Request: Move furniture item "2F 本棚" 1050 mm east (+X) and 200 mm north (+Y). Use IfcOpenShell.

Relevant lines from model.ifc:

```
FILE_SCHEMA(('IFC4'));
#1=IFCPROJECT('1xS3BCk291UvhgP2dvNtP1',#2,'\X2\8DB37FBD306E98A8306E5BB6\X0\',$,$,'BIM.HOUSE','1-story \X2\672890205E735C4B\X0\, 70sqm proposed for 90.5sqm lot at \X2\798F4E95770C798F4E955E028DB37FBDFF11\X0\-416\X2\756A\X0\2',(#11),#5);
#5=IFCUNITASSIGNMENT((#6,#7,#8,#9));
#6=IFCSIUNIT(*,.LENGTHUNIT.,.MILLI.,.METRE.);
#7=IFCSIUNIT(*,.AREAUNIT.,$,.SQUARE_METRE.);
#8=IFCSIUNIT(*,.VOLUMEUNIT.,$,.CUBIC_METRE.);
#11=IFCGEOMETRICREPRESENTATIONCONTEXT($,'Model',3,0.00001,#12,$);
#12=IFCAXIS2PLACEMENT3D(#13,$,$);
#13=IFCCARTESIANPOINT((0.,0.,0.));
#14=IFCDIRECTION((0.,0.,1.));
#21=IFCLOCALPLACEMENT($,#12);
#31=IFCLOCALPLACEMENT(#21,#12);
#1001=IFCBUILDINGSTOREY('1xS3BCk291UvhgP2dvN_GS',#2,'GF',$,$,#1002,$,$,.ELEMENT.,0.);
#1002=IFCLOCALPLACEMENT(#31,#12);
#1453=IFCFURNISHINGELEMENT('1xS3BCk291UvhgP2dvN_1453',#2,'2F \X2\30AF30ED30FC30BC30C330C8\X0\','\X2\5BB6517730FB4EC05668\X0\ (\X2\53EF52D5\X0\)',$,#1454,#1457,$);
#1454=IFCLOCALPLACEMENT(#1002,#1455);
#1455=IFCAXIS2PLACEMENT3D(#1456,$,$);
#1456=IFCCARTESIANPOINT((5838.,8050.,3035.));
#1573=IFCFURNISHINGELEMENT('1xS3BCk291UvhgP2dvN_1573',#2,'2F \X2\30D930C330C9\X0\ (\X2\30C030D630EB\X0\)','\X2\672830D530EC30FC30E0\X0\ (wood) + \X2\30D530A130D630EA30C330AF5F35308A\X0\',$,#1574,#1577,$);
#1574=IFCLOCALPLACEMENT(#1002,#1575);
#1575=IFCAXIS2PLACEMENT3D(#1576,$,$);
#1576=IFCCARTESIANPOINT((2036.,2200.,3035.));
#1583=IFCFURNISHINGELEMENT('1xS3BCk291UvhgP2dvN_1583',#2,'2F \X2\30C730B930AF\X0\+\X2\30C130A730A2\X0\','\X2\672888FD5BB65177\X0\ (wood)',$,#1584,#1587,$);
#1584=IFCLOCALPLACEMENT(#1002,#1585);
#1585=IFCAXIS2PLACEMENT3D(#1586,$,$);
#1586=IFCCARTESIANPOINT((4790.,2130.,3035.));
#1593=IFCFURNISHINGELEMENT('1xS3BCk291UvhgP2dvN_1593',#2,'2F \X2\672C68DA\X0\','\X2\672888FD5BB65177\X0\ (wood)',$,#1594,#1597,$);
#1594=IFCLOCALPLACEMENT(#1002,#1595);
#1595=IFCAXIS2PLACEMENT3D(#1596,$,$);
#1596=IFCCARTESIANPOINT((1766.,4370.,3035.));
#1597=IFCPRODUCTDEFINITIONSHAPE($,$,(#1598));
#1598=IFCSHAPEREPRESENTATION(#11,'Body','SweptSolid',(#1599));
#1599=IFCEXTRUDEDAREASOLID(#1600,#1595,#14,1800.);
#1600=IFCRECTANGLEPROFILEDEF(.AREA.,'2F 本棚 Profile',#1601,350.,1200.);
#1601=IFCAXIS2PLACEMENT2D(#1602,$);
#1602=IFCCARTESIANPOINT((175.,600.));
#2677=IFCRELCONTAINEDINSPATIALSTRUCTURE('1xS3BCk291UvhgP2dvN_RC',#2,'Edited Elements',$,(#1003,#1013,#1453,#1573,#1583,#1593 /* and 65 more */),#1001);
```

```python
import ifcopenshell
import ifcopenshell.api.geometry
import ifcopenshell.util.placement
import ifcopenshell.util.unit

model = ifcopenshell.open("model.ifc")
unit_scale = ifcopenshell.util.unit.calculate_unit_scale(model)

item = model.by_guid("1xS3BCk291UvhgP2dvN_1593")
matrix = ifcopenshell.util.placement.get_local_placement(item.ObjectPlacement)
matrix[0, 3] += 1.05 / unit_scale
matrix[1, 3] += 0.2 / unit_scale
ifcopenshell.api.geometry.edit_object_placement(model, product=item, matrix=matrix, is_si=False)

print(ifcopenshell.util.placement.get_local_placement(item.ObjectPlacement).round(3) + 0.0)

model.write("model_edited.ifc")
```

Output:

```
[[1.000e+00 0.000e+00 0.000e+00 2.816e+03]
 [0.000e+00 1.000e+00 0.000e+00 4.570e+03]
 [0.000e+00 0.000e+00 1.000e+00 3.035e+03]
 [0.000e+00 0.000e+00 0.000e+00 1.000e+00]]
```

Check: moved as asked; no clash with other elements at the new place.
